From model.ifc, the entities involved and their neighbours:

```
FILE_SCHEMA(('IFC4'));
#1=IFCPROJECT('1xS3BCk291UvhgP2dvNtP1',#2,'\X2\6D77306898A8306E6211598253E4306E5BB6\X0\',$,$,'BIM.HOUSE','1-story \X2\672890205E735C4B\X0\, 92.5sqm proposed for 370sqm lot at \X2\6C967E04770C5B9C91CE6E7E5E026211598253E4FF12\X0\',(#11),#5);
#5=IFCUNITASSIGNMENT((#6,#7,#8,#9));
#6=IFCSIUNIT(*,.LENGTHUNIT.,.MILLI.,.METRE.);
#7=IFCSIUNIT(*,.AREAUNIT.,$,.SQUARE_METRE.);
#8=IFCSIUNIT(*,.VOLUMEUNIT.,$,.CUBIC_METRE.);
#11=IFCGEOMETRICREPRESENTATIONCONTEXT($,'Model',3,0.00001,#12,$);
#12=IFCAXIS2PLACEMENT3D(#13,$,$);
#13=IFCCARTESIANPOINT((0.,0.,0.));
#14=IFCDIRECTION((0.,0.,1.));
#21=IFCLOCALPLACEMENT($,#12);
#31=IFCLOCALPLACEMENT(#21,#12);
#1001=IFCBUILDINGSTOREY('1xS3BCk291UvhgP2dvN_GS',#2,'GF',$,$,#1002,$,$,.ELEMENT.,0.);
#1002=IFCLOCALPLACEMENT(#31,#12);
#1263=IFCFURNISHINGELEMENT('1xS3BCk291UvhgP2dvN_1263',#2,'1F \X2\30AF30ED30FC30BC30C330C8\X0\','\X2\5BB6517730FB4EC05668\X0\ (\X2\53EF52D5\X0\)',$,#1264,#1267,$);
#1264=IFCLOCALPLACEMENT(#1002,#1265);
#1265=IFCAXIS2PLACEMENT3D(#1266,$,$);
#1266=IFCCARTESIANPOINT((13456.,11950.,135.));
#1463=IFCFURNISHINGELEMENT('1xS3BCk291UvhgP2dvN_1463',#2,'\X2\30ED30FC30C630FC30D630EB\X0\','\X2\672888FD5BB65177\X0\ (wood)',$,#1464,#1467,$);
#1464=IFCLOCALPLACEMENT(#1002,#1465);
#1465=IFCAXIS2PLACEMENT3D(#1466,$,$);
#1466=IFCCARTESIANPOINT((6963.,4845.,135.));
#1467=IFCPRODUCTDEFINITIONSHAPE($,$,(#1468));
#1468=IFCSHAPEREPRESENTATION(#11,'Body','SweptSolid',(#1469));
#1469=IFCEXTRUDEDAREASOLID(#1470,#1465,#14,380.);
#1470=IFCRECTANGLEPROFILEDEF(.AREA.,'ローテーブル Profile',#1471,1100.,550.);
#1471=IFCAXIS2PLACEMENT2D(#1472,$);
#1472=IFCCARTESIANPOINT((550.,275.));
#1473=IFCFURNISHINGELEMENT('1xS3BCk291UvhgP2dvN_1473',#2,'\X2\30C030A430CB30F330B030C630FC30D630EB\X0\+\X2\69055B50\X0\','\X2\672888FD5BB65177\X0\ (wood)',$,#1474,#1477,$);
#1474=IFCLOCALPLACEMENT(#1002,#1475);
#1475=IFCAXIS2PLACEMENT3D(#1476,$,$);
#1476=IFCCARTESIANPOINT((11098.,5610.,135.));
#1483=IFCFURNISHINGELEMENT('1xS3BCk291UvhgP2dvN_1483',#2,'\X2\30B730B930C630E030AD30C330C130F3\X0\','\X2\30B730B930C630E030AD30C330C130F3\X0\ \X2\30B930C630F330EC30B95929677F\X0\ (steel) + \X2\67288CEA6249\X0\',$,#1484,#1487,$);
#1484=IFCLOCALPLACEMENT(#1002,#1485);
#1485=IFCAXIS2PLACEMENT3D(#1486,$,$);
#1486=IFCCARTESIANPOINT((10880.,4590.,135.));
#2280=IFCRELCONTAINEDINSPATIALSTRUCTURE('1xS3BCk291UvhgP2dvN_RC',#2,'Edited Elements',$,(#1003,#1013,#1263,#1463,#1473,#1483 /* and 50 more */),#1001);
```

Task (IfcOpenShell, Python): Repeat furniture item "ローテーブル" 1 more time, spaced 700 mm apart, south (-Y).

```python
import numpy as np
import ifcopenshell
import ifcopenshell.api.geometry
import ifcopenshell.api.root
import ifcopenshell.util.element
import ifcopenshell.util.placement

model = ifcopenshell.open("model.ifc")


def reuse_history(source, copy):
    """copy_class also copies each property set's owner history, people and application; keep the originals."""
    for rel in copy.IsDefinedBy:
        if rel.is_a("IfcRelDefinesByProperties") and (history := rel.RelatingPropertyDefinition.OwnerHistory):
            rel.RelatingPropertyDefinition.OwnerHistory = source.OwnerHistory
            ifcopenshell.util.element.remove_deep2(model, history)


source = model.by_guid("1xS3BCk291UvhgP2dvN_1463")
base = ifcopenshell.util.placement.get_local_placement(source.ObjectPlacement)
step = np.array([0.0, -1.0, 0.0]) * 700.0

for i in range(1, 2):
    copy = ifcopenshell.api.root.copy_class(model, product=source)
    copy.Representation = ifcopenshell.util.element.copy_deep(
        model, source.Representation, exclude=["IfcGeometricRepresentationContext", "IfcRepresentationMap"]
    )
    reuse_history(source, copy)
    matrix = base.copy()
    matrix[:3, 3] += i * step
    print("added at", matrix[:3, 3].round(3) + 0.0)
    ifcopenshell.api.geometry.edit_object_placement(model, product=copy, matrix=matrix, is_si=False)

model.write("model_v2.ifc")
```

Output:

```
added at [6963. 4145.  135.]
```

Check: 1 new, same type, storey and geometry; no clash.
